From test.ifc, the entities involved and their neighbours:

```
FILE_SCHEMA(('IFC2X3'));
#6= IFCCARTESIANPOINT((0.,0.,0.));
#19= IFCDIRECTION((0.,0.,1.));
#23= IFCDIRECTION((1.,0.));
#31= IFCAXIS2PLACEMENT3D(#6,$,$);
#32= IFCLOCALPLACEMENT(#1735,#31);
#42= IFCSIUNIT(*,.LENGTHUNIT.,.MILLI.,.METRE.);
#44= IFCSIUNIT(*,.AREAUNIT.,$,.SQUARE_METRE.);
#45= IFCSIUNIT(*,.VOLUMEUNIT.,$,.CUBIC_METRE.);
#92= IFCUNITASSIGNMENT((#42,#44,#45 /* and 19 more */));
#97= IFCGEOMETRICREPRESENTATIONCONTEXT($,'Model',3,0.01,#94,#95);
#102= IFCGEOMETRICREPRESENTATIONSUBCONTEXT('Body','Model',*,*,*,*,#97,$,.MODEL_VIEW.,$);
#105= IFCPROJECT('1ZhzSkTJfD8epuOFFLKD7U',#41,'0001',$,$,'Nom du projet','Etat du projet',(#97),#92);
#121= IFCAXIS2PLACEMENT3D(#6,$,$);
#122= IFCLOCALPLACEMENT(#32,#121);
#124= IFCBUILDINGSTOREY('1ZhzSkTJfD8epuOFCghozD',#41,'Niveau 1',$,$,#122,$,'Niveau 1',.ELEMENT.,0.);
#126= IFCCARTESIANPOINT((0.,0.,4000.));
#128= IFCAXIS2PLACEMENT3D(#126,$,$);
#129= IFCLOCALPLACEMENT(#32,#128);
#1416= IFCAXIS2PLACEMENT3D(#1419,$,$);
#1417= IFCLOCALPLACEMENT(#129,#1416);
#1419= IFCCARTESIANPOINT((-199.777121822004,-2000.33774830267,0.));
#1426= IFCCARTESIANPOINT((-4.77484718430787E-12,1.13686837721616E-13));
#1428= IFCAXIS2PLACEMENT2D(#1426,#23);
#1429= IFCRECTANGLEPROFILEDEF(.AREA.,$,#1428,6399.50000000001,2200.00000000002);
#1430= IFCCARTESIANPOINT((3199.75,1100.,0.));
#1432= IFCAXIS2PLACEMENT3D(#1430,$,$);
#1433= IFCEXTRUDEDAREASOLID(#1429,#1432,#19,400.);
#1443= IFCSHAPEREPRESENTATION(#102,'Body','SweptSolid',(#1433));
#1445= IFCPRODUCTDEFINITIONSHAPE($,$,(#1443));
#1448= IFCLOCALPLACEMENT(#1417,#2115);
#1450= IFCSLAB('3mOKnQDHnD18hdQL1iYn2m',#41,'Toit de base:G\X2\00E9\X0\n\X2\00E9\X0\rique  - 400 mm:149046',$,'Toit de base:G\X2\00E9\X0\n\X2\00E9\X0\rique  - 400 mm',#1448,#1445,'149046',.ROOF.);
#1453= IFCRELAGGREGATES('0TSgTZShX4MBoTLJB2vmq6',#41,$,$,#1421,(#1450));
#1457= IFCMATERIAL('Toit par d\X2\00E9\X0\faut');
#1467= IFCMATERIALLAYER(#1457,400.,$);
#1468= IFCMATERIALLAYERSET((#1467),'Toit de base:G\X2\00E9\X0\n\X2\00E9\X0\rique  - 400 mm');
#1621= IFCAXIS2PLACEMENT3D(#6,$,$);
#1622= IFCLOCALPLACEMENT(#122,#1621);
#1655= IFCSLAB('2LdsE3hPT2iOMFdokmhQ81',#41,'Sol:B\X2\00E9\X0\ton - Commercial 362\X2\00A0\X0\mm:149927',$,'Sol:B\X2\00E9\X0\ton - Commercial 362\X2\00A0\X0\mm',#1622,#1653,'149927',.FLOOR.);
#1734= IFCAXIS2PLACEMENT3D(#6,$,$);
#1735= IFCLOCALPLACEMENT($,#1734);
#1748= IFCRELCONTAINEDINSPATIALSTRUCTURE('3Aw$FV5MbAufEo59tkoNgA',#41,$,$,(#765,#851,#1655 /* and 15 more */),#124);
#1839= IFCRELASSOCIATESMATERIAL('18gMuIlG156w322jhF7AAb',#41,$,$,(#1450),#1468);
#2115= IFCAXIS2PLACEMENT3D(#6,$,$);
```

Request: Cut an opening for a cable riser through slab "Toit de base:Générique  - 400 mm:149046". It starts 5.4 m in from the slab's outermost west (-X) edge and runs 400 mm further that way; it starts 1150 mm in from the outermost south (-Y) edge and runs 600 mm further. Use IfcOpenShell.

```python
import numpy as np
import ifcopenshell
import ifcopenshell.api.feature
import ifcopenshell.api.geometry
import ifcopenshell.api.root
import ifcopenshell.geom
import ifcopenshell.util.placement
import ifcopenshell.util.representation
import ifcopenshell.util.shape
import ifcopenshell.util.unit

model = ifcopenshell.open("test.ifc")
unit_scale = ifcopenshell.util.unit.calculate_unit_scale(model)
settings = ifcopenshell.geom.settings()


def volume(element):
    """Net volume in cubic metres, openings subtracted."""
    shape = ifcopenshell.geom.create_shape(settings, element)
    return ifcopenshell.util.shape.get_volume(shape.geometry)


slab = model.by_guid("3mOKnQDHnD18hdQL1iYn2m")
before = volume(slab)

# Extent in the slab's own axes, in metres. The edges named are its -X and -Y sides.
slab_shape = ifcopenshell.geom.create_shape(settings, slab)
vertices = ifcopenshell.util.shape.get_vertices(slab_shape.geometry)
x_min, y_min, bottom = vertices.min(axis=0)
top = vertices[:, 2].max()

opening = ifcopenshell.api.root.create_entity(model, ifc_class="IfcOpeningElement", name="Cable riser opening")
context = ifcopenshell.util.representation.get_context(model, "Model", "Body", "MODEL_VIEW")
width, depth = 0.4, 0.6
outline = [(0.0, 0.0), (width, 0.0), (width, depth), (0.0, depth), (0.0, 0.0)]
# Overshoot both faces by 50 mm so the cut is clean.
shape = ifcopenshell.api.geometry.add_slab_representation(
    model, context=context, depth=top - bottom + 0.1, polyline=outline
)
ifcopenshell.api.geometry.assign_representation(model, product=opening, representation=shape)

matrix = ifcopenshell.util.placement.get_local_placement(slab.ObjectPlacement)
matrix[:, 3] = matrix @ np.append(np.array([x_min + 5.4, y_min + 1.15, bottom - 0.05]) / unit_scale, 1.0)
ifcopenshell.api.geometry.edit_object_placement(model, product=opening, matrix=matrix, is_si=False)
ifcopenshell.api.feature.add_feature(model, feature=opening, element=slab)

after = volume(slab)

print(f"slab volume {before:.3f} -> {after:.3f} m3")

model.write("test-out.ifc")
```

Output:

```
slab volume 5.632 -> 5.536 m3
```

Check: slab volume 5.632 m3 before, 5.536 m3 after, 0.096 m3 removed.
